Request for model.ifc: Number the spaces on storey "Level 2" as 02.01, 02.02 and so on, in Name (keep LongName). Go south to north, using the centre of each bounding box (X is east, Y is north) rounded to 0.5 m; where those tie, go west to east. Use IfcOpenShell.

First a look at what the model holds.

```python
import ifcopenshell
import ifcopenshell.util.element
import ifcopenshell.util.placement

model = ifcopenshell.open("model.ifc")
print(model.schema)
storey = next(s for s in model.by_type("IfcBuildingStorey") if s.Name == "Level 2")
spaces = [e for e in ifcopenshell.util.element.get_decomposition(storey) if e.is_a("IfcSpace")]
for e in sorted(spaces, key=lambda e: e.id()):
    origin = ifcopenshell.util.placement.get_local_placement(e.ObjectPlacement)[:3, 3]
    print(e.id(), e.Name, e.LongName, origin.round(2) + 0.0, sep=" | ")
```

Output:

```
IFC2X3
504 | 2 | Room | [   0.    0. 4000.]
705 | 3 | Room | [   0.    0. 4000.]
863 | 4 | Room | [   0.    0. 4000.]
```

```python
import ifcopenshell
import ifcopenshell.geom
import ifcopenshell.util.element
import ifcopenshell.util.shape

model = ifcopenshell.open("model.ifc")
settings = ifcopenshell.geom.settings()
settings.set("use-world-coords", True)


def centre(element):
    shape = ifcopenshell.geom.create_shape(settings, element)
    return ifcopenshell.util.shape.get_bbox_centroid(shape.geometry)


storey = next(s for s in model.by_type("IfcBuildingStorey") if s.Name == "Level 2")
spaces = [e for e in ifcopenshell.util.element.get_decomposition(storey) if e.is_a("IfcSpace")]

# Insertion points can sit at a corner or the storey origin, so sort by the geometry (in metres).
centres = {e: centre(e) for e in spaces}
spaces.sort(key=lambda e: (round(centres[e][1] / 0.5), centres[e][0]))

for i, e in enumerate(spaces, start=1):
    number = f"02.{i:02d}"
    e.Name = number
    print(e.id(), number)

model.write("model_rev.ifc")
```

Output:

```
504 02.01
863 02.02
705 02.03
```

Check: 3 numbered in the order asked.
